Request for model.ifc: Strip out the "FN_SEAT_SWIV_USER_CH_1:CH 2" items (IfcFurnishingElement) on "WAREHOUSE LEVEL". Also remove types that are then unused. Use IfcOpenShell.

First a look at what the model holds.

```python
import ifcopenshell
import ifcopenshell.util.element

model = ifcopenshell.open("model.ifc")
print(model.schema)
storey = next(s for s in model.by_type("IfcBuildingStorey") if s.Name == "WAREHOUSE LEVEL")
furniture = [e for e in ifcopenshell.util.element.get_decomposition(storey) if e.is_a("IfcFurnishingElement")]
seen = {}
for e in furniture:
    element_type = ifcopenshell.util.element.get_type(e)
    name = element_type.Name if element_type not in (None, e) else None
    seen[name] = seen.get(name, 0) + 1
for name, count in sorted(seen.items(), key=str):
    print(count, "x", name)
```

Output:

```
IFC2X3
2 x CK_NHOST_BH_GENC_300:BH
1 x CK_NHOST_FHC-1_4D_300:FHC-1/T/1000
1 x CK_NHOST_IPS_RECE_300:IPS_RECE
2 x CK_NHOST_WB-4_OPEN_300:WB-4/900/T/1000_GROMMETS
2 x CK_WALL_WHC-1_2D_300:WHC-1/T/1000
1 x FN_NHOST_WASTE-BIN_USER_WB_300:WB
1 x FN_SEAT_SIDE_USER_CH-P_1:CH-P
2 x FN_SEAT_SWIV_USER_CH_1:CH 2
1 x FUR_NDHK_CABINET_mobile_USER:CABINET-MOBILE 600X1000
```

```python
import ifcopenshell
import ifcopenshell.api.root
import ifcopenshell.util.element

model = ifcopenshell.open("model.ifc")

storey = next(s for s in model.by_type("IfcBuildingStorey") if s.Name == "WAREHOUSE LEVEL")
furniture = [e for e in ifcopenshell.util.element.get_decomposition(storey) if e.is_a("IfcFurnishingElement")]
targets = [e for e in furniture if (t := ifcopenshell.util.element.get_type(e)) not in (None, e) and t.Name == "FN_SEAT_SWIV_USER_CH_1:CH 2"]
types = {ifcopenshell.util.element.get_type(e) for e in targets} - {None, *targets}

for e in targets:
    ifcopenshell.api.root.remove_product(model, product=e)
print(len(targets), "removed")

unused = [t for t in types if not ifcopenshell.util.element.get_types(t)]
for t in unused:
    ifcopenshell.api.root.remove_product(model, product=t)
print(len(unused), "unused types removed")

model.write("model-out.ifc")
```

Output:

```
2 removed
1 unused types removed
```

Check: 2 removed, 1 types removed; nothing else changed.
